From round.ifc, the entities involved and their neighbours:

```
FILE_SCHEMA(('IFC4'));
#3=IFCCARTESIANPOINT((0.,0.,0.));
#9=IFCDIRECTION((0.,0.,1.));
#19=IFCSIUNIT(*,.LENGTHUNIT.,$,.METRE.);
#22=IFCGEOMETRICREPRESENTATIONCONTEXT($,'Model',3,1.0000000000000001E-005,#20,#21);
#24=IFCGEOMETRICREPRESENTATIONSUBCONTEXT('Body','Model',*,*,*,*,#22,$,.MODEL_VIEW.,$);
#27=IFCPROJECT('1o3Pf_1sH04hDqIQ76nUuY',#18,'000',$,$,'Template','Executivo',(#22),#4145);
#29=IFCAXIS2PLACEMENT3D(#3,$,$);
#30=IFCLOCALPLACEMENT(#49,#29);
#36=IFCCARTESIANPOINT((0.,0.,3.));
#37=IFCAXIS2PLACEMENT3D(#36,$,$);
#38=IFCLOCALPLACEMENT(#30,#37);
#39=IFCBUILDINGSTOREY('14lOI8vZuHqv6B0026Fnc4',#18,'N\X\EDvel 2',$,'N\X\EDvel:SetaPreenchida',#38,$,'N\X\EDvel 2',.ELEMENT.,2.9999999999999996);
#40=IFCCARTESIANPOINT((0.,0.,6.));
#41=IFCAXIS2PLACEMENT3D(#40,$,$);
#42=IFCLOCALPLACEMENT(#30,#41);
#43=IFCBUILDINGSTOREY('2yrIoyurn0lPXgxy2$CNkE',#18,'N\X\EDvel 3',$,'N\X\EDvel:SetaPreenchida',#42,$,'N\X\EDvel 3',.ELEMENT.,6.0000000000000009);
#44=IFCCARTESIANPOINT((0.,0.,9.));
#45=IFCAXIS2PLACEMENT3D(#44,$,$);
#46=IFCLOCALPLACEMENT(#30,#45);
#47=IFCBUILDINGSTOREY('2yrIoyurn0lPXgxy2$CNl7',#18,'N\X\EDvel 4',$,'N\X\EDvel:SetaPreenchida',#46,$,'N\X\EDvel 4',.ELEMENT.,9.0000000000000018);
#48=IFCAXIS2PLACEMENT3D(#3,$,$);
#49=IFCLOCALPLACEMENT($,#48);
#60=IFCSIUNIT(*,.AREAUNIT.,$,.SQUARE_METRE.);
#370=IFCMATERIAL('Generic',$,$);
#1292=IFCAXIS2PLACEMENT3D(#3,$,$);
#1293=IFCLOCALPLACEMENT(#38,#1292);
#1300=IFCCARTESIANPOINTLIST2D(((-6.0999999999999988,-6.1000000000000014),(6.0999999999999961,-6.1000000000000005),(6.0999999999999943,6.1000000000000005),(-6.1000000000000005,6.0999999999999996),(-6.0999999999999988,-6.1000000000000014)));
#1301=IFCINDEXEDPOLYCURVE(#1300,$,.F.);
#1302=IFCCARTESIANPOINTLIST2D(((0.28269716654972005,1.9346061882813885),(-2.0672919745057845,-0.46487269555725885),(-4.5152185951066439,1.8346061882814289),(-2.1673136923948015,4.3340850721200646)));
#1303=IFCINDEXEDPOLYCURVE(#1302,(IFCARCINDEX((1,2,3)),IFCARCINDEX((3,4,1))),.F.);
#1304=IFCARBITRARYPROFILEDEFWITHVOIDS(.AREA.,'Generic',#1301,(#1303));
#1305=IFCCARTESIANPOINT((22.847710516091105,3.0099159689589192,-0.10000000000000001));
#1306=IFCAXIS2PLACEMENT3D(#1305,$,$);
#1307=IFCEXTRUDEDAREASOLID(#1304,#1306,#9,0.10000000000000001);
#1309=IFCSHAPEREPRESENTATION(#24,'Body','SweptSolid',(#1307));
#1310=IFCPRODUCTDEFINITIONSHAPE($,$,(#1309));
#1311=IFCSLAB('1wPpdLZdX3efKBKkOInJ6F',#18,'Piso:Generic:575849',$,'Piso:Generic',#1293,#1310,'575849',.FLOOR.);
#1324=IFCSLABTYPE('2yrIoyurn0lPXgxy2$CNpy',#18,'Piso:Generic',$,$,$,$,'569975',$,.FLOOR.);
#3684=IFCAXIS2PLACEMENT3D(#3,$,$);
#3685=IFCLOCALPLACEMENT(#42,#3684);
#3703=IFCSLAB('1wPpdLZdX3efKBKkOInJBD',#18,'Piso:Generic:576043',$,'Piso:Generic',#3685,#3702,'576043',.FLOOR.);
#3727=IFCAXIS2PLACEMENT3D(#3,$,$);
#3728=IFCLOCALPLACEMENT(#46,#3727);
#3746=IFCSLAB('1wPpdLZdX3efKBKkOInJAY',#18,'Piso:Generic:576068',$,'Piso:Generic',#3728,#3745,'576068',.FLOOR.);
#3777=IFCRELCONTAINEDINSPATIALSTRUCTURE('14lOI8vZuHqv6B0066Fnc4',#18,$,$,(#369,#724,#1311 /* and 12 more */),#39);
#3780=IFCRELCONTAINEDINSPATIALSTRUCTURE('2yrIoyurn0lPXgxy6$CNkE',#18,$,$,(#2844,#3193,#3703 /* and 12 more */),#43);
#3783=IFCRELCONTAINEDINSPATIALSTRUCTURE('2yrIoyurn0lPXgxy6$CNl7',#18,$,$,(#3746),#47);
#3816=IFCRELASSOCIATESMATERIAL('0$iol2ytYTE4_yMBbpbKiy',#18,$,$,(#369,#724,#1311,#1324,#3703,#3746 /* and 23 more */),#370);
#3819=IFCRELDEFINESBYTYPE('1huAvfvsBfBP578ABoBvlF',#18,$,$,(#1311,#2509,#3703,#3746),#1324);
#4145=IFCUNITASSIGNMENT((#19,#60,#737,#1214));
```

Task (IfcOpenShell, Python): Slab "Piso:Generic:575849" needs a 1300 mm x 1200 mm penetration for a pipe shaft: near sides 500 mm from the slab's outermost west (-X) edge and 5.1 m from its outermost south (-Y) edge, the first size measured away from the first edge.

```python
import numpy as np
import ifcopenshell
import ifcopenshell.api.feature
import ifcopenshell.api.geometry
import ifcopenshell.api.root
import ifcopenshell.geom
import ifcopenshell.util.placement
import ifcopenshell.util.representation
import ifcopenshell.util.shape
import ifcopenshell.util.unit

model = ifcopenshell.open("round.ifc")
unit_scale = ifcopenshell.util.unit.calculate_unit_scale(model)
settings = ifcopenshell.geom.settings()


def volume(element):
    """Net volume in cubic metres, openings subtracted."""
    shape = ifcopenshell.geom.create_shape(settings, element)
    return ifcopenshell.util.shape.get_volume(shape.geometry)


slab = model.by_guid("1wPpdLZdX3efKBKkOInJ6F")
before = volume(slab)

# Extent in the slab's own axes, in metres. The edges named are its -X and -Y sides.
slab_shape = ifcopenshell.geom.create_shape(settings, slab)
vertices = ifcopenshell.util.shape.get_vertices(slab_shape.geometry)
x_min, y_min, bottom = vertices.min(axis=0)
top = vertices[:, 2].max()

opening = ifcopenshell.api.root.create_entity(model, ifc_class="IfcOpeningElement", name="Pipe shaft opening", predefined_type="OPENING")
context = ifcopenshell.util.representation.get_context(model, "Model", "Body", "MODEL_VIEW")
width, depth = 1.3, 1.2
outline = [(0.0, 0.0), (width, 0.0), (width, depth), (0.0, depth), (0.0, 0.0)]
# Overshoot both faces by 50 mm so the cut is clean.
shape = ifcopenshell.api.geometry.add_slab_representation(
    model, context=context, depth=top - bottom + 0.1, polyline=outline
)
ifcopenshell.api.geometry.assign_representation(model, product=opening, representation=shape)

matrix = ifcopenshell.util.placement.get_local_placement(slab.ObjectPlacement)
matrix[:, 3] = matrix @ np.append(np.array([x_min + 0.5, y_min + 5.1, bottom - 0.05]) / unit_scale, 1.0)
ifcopenshell.api.geometry.edit_object_placement(model, product=opening, matrix=matrix, is_si=False)
ifcopenshell.api.feature.add_feature(model, feature=opening, element=slab)

after = volume(slab)

print(f"slab volume {before:.3f} -> {after:.3f} m3")

model.write("round_updated.ifc")
```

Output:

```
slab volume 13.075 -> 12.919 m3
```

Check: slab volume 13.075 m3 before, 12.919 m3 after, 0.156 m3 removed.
